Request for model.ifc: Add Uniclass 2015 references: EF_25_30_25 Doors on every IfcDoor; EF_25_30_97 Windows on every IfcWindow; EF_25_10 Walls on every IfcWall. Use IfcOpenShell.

First a look at what the model holds.

```python
import ifcopenshell

model = ifcopenshell.open("model.ifc")
print(model.schema)
print("classifications:", [c.Name for c in model.by_type("IfcClassification")])
for ifc_class in ("IfcDoor", "IfcRoof", "IfcStair", "IfcWall", "IfcWindow"):
    print(ifc_class, len(model.by_type(ifc_class)))
```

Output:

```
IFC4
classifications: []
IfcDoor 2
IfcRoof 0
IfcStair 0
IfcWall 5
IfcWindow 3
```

```python
import ifcopenshell
import ifcopenshell.api.classification

model = ifcopenshell.open("model.ifc")

system = ifcopenshell.api.classification.add_classification(model, classification="Uniclass 2015")

codes = {
    "IfcDoor": ("EF_25_30_25", "Doors"),
    "IfcWindow": ("EF_25_30_97", "Windows"),
    "IfcWall": ("EF_25_10", "Walls"),
}
for ifc_class, (code, name) in codes.items():
    products = model.by_type(ifc_class)
    ifcopenshell.api.classification.add_reference(
        model, products=products, classification=system, identification=code, name=name
    )
    print(code, len(products))

model.write("model-out.ifc")
```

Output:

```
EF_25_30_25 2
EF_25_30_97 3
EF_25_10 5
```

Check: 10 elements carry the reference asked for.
